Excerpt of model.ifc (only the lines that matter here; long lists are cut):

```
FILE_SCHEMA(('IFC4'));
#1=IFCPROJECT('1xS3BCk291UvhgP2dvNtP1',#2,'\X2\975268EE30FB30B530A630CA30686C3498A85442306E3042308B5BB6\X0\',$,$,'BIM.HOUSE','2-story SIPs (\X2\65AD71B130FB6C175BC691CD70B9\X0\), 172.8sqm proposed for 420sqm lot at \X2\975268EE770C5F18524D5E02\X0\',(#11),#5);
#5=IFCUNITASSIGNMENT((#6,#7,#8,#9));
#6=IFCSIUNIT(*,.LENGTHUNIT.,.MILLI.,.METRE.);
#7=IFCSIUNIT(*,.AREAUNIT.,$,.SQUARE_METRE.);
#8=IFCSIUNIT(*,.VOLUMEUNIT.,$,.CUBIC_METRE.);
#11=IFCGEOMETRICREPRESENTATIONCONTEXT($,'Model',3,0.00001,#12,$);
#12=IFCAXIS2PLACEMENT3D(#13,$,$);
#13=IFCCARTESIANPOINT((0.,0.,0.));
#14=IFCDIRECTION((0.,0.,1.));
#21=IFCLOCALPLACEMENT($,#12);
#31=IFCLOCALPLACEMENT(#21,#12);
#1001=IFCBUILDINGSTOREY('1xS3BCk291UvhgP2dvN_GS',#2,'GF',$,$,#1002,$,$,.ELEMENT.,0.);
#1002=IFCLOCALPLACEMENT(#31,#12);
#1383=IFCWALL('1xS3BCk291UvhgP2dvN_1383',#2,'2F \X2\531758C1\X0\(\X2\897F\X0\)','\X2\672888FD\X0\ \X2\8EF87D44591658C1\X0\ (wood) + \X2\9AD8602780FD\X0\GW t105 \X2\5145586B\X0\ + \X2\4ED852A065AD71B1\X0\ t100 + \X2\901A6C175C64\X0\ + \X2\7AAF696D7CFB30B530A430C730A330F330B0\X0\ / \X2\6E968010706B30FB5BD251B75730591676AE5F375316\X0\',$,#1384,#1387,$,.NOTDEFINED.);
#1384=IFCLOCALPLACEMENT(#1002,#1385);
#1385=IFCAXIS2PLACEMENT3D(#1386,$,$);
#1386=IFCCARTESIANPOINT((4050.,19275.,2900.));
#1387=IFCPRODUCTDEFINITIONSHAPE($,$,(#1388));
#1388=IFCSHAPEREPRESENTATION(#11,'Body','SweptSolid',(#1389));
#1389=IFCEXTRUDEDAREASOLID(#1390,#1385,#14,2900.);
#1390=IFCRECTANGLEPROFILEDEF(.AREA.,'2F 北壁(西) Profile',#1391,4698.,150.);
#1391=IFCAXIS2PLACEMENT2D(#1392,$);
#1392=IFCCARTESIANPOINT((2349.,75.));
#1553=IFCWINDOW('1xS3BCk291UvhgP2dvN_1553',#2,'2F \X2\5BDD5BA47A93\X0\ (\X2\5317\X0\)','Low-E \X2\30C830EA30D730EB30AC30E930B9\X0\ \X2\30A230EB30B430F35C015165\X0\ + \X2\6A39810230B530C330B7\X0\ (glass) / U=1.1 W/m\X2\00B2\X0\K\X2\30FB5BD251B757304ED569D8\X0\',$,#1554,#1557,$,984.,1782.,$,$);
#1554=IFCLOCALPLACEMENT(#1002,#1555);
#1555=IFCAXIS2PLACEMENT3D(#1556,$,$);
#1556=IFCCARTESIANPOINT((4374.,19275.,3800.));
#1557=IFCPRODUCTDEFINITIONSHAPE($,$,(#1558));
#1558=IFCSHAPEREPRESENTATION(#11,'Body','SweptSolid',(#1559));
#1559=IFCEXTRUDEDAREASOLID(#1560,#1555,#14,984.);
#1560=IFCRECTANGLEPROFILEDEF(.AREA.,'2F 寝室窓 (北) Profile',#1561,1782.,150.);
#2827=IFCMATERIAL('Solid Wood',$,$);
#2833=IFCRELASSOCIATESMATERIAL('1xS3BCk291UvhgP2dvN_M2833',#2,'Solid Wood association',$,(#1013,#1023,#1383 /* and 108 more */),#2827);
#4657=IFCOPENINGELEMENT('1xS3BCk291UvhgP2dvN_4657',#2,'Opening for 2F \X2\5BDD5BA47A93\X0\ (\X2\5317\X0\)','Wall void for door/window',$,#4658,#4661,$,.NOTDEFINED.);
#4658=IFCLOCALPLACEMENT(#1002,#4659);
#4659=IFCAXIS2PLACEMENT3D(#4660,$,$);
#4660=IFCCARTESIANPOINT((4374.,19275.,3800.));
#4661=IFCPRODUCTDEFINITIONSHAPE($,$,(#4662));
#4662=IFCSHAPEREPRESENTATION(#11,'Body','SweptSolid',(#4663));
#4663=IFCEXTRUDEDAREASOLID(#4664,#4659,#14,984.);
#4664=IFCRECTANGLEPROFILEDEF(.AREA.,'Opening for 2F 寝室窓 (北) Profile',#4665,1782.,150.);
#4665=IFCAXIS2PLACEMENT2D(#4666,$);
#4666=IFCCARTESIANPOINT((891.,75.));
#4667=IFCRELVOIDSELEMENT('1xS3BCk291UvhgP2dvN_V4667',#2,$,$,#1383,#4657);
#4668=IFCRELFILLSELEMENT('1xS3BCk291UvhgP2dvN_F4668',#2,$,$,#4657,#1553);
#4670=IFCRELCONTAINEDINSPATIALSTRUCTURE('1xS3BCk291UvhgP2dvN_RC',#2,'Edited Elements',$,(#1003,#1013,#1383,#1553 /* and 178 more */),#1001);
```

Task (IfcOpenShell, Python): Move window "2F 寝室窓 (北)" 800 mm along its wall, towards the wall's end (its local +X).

```python
import ifcopenshell
import ifcopenshell.api.geometry
import ifcopenshell.util.placement
import ifcopenshell.util.unit

model = ifcopenshell.open("model.ifc")
unit_scale = ifcopenshell.util.unit.calculate_unit_scale(model)

window = model.by_guid("1xS3BCk291UvhgP2dvN_1553")
opening = window.FillsVoids[0].RelatingOpeningElement
wall = opening.VoidsElements[0].RelatingBuildingElement

wall_matrix = ifcopenshell.util.placement.get_local_placement(wall.ObjectPlacement)
shift = wall_matrix[:3, 0] * 0.8 / unit_scale
before = ifcopenshell.util.placement.get_local_placement(window.ObjectPlacement)[:3, 3].copy()

# The window is not placed relative to its opening, so move both.
for product in (opening, window):
    matrix = ifcopenshell.util.placement.get_local_placement(product.ObjectPlacement)
    matrix[:3, 3] += shift
    ifcopenshell.api.geometry.edit_object_placement(model, product=product, matrix=matrix, is_si=False)

after = ifcopenshell.util.placement.get_local_placement(window.ObjectPlacement)[:3, 3]
print("window moved by", (after - before).round(3) + 0.0)

model.write("model_v2.ifc")
```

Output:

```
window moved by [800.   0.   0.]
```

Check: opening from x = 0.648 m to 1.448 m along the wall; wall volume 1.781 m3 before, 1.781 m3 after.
